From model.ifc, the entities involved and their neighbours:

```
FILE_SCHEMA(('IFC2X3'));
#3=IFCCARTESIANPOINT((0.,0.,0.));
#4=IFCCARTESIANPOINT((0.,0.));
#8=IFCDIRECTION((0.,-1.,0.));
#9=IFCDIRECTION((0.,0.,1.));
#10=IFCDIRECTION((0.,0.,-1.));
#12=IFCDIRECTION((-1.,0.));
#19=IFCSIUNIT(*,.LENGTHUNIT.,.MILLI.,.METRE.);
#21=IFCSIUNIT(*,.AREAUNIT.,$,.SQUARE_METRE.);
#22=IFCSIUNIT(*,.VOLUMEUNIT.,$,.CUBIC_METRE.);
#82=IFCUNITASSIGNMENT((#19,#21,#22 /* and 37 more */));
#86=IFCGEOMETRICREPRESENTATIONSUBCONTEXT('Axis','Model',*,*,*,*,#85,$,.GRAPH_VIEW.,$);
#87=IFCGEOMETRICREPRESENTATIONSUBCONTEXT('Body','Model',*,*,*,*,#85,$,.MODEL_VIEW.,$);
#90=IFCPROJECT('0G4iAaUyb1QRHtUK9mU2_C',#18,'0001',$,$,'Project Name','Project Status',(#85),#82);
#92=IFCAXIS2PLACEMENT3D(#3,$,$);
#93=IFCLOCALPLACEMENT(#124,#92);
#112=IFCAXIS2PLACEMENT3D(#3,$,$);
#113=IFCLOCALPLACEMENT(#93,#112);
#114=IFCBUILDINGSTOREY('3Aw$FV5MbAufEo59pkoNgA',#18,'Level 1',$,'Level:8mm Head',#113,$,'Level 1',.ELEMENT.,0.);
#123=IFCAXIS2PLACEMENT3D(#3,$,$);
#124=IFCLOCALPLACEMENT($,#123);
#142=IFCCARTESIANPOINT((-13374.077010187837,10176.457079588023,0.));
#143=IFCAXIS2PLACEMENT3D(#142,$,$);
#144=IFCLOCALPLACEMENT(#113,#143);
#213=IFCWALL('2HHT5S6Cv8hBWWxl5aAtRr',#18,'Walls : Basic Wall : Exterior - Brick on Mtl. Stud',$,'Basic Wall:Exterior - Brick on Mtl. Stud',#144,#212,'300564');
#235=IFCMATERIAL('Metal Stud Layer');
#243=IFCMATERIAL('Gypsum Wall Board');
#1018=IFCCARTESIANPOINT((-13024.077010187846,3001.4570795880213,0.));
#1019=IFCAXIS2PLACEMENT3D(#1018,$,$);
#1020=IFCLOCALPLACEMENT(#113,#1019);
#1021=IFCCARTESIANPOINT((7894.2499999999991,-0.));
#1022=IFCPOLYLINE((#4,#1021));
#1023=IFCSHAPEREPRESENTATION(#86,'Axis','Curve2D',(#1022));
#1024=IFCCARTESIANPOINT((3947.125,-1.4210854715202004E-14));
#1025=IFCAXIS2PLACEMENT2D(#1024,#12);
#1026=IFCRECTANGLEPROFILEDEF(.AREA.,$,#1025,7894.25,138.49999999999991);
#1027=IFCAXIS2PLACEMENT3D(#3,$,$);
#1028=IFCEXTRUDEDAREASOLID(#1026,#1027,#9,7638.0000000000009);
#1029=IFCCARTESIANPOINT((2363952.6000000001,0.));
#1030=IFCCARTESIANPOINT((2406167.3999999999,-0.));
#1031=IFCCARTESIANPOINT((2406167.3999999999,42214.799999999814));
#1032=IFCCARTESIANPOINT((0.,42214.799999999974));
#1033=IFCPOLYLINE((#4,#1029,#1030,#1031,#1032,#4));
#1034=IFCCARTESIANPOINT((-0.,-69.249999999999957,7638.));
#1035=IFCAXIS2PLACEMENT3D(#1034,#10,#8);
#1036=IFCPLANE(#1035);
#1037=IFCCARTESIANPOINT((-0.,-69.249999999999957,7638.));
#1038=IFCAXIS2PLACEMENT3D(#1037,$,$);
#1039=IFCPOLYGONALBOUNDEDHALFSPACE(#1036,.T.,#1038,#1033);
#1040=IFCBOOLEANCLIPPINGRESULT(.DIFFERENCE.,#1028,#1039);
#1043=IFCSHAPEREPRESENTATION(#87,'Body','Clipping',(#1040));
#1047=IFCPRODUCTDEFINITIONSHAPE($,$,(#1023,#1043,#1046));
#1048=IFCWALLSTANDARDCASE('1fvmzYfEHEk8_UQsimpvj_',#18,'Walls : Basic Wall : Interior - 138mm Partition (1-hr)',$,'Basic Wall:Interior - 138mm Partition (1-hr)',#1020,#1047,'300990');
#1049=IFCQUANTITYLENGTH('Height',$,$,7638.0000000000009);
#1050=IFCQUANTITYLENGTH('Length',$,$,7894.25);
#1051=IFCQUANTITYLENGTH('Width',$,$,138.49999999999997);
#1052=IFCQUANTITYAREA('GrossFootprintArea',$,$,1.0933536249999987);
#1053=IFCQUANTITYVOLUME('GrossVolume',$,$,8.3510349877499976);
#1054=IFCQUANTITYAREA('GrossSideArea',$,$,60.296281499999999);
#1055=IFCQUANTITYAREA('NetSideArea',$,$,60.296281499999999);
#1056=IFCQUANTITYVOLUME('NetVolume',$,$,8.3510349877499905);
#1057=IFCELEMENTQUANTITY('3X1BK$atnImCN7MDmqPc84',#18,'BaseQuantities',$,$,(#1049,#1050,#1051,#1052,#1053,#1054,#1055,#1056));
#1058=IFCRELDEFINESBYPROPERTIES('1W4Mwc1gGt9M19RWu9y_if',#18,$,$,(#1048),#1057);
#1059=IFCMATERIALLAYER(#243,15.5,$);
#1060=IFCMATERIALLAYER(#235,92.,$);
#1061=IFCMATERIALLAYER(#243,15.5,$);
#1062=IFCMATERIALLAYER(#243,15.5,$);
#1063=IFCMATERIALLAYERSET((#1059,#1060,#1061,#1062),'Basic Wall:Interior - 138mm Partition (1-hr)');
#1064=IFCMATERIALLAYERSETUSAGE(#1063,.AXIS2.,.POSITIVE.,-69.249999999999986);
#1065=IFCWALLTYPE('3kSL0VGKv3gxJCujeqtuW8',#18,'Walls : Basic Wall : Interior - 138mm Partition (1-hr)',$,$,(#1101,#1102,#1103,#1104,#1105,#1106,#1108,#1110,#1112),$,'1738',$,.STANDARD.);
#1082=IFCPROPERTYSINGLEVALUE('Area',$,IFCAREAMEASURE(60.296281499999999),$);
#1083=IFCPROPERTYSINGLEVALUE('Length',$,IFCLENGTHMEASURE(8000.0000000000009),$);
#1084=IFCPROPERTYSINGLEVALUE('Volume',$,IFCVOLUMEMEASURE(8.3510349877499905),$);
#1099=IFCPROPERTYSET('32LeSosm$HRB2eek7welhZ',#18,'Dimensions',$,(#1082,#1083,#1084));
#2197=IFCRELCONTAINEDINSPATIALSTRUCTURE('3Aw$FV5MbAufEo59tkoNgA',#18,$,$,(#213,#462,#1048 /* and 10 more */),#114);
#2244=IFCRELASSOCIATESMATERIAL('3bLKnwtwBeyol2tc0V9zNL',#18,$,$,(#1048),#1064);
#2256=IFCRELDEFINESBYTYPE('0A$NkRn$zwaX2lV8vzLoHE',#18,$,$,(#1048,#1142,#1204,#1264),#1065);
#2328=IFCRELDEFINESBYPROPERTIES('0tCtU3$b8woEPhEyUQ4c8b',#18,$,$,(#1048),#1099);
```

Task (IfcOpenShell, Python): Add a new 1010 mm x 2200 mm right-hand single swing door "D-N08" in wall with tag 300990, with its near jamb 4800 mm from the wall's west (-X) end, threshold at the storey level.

```python
import numpy as np
import ifcopenshell
import ifcopenshell.api.feature
import ifcopenshell.api.geometry
import ifcopenshell.api.pset
import ifcopenshell.api.root
import ifcopenshell.api.spatial
import ifcopenshell.api.type
import ifcopenshell.geom
import ifcopenshell.util.element
import ifcopenshell.util.placement
import ifcopenshell.util.representation
import ifcopenshell.util.shape
import ifcopenshell.util.unit

model = ifcopenshell.open("model.ifc")
unit_scale = ifcopenshell.util.unit.calculate_unit_scale(model)
area_scale = ifcopenshell.util.unit.calculate_unit_scale(model, "AREAUNIT")
volume_scale = ifcopenshell.util.unit.calculate_unit_scale(model, "VOLUMEUNIT")
settings = ifcopenshell.geom.settings()


def volume(element):
    """Net volume in cubic metres, openings subtracted."""
    shape = ifcopenshell.geom.create_shape(settings, element)
    return ifcopenshell.util.shape.get_volume(shape.geometry)


wall = model.by_guid("1fvmzYfEHEk8_UQsimpvj_")
storey = ifcopenshell.util.element.get_container(wall, ifc_class="IfcBuildingStorey")
context = ifcopenshell.util.representation.get_context(model, "Model", "Body", "MODEL_VIEW")
before = volume(wall)

width, height, from_end, sill = 1.01, 2.2, 4.8, 0.0  # metres

# The wall runs along its own X axis, and the end named is its -X end.
wall_shape = ifcopenshell.geom.create_shape(settings, wall)
x, y, z = ifcopenshell.util.shape.get_vertices(wall_shape.geometry).T
start = x.min() + from_end
face, thickness = float(y.min()), float(y.max() - y.min())
wall_matrix = ifcopenshell.util.placement.get_local_placement(wall.ObjectPlacement)
level = ifcopenshell.util.placement.get_local_placement(storey.ObjectPlacement)[2, 3]


def in_wall(x, y):
    """Placement at x, y metres in the wall's axes, at sill height."""
    matrix = wall_matrix.copy()
    matrix[:, 3] = wall_matrix @ np.array([x / unit_scale, y / unit_scale, 0.0, 1.0])
    matrix[2, 3] = level + sill / unit_scale
    return matrix


# Opening: a box that overshoots both wall faces by 50 mm.
opening = ifcopenshell.api.root.create_entity(model, ifc_class="IfcOpeningElement")
box = ifcopenshell.api.geometry.add_wall_representation(
    model, context=context, length=width, height=height, thickness=thickness + 0.1
)
ifcopenshell.api.geometry.assign_representation(model, product=opening, representation=box)
ifcopenshell.api.geometry.edit_object_placement(model, product=opening, matrix=in_wall(start, face - 0.05), is_si=False)
ifcopenshell.api.feature.add_feature(model, feature=opening, element=wall)

door = ifcopenshell.api.root.create_entity(model, ifc_class="IfcDoor", name="D-N08")
door.OverallWidth, door.OverallHeight = width / unit_scale, height / unit_scale
body = ifcopenshell.api.geometry.add_door_representation(
    model,
    context=context,
    overall_width=door.OverallWidth,
    overall_height=door.OverallHeight,
    operation_type="SINGLE_SWING_RIGHT",
    lining_properties={"LiningDepth": thickness / unit_scale, "ThresholdDepth": thickness / unit_scale},
)
ifcopenshell.api.geometry.assign_representation(model, product=door, representation=body)
ifcopenshell.api.spatial.assign_container(model, products=[door], relating_structure=storey)
fills = ifcopenshell.api.feature.add_filling(model, opening=opening, element=door)
fills.OwnerHistory = door.OwnerHistory  # required in IFC2X3

# IFC2X3 keeps the operation on the door style.
style = ifcopenshell.api.root.create_entity(model, ifc_class="IfcDoorStyle", name="D-N08")
style.OperationType, style.ConstructionType = "SINGLE_SWING_RIGHT", "NOTDEFINED"
style.ParameterTakesPrecedence = style.Sizeable = False
ifcopenshell.api.type.assign_type(model, related_objects=[door], relating_type=style)

# The lining spans the wall, so the door starts at the wall face.
ifcopenshell.api.geometry.edit_object_placement(model, product=door, matrix=in_wall(start, face), is_si=False)

after = volume(wall)

# Update the wall's stored quantities.
qto = model.by_id(ifcopenshell.util.element.get_pset(wall, "BaseQuantities", should_inherit=False)["id"])
ifcopenshell.api.pset.edit_qto(model, qto=qto, properties={
    "NetSideArea": after / thickness / area_scale,
    "NetVolume": after / volume_scale,
})
pset = model.by_id(ifcopenshell.util.element.get_pset(wall, "Dimensions", should_inherit=False)["id"])
ifcopenshell.api.pset.edit_pset(model, pset=pset, properties={
    "Area": model.create_entity("IfcAreaMeasure", after / thickness / area_scale),
    "Volume": model.create_entity("IfcVolumeMeasure", after / volume_scale),
})

print(f"wall volume {before:.3f} -> {after:.3f} m3")

model.write("model_rev.ifc")
```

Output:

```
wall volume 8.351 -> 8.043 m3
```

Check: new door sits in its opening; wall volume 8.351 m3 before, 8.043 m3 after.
